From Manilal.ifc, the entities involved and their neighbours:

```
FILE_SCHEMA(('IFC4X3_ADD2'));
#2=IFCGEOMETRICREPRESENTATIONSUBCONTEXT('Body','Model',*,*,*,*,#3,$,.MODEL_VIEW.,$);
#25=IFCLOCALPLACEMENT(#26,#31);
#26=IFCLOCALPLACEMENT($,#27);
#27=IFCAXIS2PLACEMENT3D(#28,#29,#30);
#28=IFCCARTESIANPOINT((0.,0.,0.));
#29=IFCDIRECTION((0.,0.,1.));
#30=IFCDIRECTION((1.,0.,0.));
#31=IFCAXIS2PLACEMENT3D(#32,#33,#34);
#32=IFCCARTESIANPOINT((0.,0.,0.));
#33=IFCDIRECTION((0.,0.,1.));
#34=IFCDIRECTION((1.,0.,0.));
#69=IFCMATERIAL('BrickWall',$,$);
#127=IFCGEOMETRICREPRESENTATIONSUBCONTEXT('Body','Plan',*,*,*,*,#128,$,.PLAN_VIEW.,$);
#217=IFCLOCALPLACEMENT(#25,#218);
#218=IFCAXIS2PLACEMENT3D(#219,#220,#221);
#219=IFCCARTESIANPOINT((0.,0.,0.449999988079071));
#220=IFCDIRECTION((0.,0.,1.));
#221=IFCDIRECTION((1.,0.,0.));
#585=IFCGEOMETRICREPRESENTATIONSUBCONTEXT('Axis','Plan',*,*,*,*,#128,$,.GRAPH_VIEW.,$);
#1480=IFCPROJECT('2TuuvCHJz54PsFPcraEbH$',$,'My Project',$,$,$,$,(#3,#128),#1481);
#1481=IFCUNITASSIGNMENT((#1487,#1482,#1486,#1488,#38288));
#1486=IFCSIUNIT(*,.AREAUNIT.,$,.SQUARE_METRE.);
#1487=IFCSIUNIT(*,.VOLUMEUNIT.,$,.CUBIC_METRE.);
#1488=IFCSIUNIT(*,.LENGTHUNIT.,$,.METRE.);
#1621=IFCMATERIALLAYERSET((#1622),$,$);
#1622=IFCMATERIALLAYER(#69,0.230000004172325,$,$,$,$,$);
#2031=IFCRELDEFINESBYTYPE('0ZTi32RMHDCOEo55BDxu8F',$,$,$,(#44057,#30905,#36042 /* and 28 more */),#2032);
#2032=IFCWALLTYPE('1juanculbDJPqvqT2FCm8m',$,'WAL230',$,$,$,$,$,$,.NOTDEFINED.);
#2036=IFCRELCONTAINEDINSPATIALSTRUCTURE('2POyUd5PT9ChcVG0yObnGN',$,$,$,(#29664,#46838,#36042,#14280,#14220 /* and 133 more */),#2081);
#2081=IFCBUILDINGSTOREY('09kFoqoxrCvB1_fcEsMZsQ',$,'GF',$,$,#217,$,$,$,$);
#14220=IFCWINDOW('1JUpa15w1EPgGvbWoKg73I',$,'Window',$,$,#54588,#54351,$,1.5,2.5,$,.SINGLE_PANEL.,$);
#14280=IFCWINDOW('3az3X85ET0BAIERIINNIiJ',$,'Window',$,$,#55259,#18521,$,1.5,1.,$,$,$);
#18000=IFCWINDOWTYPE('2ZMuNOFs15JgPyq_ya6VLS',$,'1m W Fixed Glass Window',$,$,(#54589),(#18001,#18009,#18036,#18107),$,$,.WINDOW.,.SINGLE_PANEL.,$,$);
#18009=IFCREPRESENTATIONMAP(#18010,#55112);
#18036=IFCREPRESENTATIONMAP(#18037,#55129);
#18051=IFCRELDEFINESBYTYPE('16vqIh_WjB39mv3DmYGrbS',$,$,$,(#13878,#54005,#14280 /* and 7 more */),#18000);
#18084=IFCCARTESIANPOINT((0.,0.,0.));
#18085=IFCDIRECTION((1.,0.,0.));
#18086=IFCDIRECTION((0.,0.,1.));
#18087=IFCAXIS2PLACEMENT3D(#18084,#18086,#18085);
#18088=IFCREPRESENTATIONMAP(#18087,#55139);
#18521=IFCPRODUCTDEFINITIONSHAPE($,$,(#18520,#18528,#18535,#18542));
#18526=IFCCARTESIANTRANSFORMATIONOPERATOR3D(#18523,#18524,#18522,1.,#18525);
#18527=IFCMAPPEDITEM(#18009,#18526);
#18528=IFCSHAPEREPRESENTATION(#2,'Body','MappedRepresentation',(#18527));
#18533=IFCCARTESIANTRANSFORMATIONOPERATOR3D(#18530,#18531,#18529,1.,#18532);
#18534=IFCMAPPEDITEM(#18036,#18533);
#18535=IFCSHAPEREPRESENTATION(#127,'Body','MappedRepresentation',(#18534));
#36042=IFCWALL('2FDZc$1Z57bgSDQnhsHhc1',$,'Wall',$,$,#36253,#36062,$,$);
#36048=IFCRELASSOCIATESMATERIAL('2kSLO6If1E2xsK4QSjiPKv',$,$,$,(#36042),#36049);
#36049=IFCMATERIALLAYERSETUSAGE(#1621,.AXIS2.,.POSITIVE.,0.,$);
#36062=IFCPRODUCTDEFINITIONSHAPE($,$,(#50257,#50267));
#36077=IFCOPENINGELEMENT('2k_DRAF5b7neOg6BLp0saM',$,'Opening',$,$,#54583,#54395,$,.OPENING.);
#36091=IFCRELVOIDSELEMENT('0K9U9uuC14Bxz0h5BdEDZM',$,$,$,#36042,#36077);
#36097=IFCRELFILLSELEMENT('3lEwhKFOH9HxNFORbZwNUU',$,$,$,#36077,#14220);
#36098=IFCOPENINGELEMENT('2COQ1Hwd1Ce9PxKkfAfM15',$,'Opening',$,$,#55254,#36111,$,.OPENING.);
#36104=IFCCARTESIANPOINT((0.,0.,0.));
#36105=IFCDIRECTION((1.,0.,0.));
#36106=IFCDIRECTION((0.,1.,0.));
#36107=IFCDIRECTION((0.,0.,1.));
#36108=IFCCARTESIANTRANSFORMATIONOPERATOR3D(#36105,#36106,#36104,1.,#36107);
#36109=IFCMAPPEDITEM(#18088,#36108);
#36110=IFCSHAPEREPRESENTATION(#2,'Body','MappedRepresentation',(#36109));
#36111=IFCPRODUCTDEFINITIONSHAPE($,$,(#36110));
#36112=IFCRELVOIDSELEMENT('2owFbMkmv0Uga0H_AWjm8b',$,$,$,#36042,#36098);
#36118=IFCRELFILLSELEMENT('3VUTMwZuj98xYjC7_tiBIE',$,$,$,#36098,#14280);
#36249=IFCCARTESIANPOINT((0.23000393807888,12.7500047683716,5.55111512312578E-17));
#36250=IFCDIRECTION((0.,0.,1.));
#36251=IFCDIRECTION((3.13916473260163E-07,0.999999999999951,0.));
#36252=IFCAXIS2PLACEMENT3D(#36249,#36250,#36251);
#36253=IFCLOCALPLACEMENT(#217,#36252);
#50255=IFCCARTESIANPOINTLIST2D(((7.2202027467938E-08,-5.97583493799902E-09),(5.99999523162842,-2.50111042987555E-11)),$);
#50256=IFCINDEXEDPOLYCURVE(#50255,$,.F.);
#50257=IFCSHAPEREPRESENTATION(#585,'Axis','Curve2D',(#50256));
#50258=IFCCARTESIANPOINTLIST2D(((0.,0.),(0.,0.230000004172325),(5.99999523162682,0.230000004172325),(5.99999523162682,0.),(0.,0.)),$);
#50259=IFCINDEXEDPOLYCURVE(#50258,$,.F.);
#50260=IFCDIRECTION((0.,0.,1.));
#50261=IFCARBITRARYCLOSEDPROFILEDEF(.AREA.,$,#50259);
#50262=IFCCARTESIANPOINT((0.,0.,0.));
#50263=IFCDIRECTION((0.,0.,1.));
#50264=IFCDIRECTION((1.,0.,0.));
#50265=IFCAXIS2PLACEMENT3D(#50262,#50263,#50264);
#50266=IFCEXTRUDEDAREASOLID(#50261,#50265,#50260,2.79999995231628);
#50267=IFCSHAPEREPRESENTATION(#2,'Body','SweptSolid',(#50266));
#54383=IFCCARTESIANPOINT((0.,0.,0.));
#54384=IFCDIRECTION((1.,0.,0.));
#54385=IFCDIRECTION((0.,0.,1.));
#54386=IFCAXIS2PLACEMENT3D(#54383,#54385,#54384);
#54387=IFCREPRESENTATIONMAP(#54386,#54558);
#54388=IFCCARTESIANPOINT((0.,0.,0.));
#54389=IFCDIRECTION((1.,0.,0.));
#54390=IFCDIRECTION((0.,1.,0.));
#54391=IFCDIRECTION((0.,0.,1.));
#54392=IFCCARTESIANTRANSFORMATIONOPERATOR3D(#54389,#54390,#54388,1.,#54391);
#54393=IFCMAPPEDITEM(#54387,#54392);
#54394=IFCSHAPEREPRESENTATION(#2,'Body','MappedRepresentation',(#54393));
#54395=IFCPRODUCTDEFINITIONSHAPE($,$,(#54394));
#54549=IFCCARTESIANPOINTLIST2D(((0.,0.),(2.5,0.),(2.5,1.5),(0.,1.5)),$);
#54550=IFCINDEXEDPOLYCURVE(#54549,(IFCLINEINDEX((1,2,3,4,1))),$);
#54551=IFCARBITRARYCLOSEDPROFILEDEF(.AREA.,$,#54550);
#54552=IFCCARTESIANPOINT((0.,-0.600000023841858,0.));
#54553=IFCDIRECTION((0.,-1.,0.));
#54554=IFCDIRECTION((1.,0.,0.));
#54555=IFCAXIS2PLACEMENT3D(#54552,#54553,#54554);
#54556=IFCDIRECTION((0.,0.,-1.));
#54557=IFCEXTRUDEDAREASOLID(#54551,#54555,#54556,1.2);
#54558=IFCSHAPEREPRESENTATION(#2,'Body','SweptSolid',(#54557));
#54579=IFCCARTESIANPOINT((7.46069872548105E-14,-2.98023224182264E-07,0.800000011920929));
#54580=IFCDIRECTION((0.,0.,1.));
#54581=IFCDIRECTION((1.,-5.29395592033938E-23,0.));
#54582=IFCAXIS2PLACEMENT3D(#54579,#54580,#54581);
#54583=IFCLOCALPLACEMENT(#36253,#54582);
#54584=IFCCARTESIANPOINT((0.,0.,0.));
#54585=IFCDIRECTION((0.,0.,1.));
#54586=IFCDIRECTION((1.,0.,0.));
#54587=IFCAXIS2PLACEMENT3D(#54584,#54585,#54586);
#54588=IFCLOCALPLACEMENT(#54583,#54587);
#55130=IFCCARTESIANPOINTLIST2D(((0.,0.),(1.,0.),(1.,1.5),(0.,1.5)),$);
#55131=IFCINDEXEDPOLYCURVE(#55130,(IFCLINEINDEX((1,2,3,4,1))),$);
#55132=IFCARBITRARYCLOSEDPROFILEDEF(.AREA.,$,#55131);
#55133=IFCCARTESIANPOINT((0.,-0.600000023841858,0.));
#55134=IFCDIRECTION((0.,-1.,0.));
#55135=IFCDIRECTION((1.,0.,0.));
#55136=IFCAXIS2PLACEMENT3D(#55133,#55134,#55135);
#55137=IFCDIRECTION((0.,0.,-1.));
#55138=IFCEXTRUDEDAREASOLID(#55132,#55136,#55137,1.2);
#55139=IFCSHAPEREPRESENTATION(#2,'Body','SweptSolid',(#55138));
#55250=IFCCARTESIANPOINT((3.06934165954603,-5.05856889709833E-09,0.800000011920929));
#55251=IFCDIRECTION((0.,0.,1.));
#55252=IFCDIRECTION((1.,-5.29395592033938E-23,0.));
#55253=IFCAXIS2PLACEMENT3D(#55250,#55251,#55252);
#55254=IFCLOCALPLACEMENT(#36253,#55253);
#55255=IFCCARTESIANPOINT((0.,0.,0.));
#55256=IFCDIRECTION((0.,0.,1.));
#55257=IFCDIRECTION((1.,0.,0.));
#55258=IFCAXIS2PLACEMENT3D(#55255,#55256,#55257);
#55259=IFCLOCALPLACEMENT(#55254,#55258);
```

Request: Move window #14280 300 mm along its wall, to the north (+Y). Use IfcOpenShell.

```python
import ifcopenshell
import ifcopenshell.api.geometry
import ifcopenshell.util.placement
import ifcopenshell.util.unit

model = ifcopenshell.open("Manilal.ifc")
unit_scale = ifcopenshell.util.unit.calculate_unit_scale(model)

window = model.by_id(14280)
opening = window.FillsVoids[0].RelatingOpeningElement
wall = opening.VoidsElements[0].RelatingBuildingElement

wall_matrix = ifcopenshell.util.placement.get_local_placement(wall.ObjectPlacement)
shift = wall_matrix[:3, 0] * 0.3 / unit_scale
before = ifcopenshell.util.placement.get_local_placement(window.ObjectPlacement)[:3, 3].copy()

# The window is placed relative to its opening, so it follows when the opening moves.
matrix = ifcopenshell.util.placement.get_local_placement(opening.ObjectPlacement)
matrix[:3, 3] += shift
ifcopenshell.api.geometry.edit_object_placement(
    model, product=opening, matrix=matrix, is_si=False, should_transform_children=True
)

after = ifcopenshell.util.placement.get_local_placement(window.ObjectPlacement)[:3, 3]
print("window moved by", (after - before).round(3) + 0.0)

model.write("Manilal_v2.ifc")
```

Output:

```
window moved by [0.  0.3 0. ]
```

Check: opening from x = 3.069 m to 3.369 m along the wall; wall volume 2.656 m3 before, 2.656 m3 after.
